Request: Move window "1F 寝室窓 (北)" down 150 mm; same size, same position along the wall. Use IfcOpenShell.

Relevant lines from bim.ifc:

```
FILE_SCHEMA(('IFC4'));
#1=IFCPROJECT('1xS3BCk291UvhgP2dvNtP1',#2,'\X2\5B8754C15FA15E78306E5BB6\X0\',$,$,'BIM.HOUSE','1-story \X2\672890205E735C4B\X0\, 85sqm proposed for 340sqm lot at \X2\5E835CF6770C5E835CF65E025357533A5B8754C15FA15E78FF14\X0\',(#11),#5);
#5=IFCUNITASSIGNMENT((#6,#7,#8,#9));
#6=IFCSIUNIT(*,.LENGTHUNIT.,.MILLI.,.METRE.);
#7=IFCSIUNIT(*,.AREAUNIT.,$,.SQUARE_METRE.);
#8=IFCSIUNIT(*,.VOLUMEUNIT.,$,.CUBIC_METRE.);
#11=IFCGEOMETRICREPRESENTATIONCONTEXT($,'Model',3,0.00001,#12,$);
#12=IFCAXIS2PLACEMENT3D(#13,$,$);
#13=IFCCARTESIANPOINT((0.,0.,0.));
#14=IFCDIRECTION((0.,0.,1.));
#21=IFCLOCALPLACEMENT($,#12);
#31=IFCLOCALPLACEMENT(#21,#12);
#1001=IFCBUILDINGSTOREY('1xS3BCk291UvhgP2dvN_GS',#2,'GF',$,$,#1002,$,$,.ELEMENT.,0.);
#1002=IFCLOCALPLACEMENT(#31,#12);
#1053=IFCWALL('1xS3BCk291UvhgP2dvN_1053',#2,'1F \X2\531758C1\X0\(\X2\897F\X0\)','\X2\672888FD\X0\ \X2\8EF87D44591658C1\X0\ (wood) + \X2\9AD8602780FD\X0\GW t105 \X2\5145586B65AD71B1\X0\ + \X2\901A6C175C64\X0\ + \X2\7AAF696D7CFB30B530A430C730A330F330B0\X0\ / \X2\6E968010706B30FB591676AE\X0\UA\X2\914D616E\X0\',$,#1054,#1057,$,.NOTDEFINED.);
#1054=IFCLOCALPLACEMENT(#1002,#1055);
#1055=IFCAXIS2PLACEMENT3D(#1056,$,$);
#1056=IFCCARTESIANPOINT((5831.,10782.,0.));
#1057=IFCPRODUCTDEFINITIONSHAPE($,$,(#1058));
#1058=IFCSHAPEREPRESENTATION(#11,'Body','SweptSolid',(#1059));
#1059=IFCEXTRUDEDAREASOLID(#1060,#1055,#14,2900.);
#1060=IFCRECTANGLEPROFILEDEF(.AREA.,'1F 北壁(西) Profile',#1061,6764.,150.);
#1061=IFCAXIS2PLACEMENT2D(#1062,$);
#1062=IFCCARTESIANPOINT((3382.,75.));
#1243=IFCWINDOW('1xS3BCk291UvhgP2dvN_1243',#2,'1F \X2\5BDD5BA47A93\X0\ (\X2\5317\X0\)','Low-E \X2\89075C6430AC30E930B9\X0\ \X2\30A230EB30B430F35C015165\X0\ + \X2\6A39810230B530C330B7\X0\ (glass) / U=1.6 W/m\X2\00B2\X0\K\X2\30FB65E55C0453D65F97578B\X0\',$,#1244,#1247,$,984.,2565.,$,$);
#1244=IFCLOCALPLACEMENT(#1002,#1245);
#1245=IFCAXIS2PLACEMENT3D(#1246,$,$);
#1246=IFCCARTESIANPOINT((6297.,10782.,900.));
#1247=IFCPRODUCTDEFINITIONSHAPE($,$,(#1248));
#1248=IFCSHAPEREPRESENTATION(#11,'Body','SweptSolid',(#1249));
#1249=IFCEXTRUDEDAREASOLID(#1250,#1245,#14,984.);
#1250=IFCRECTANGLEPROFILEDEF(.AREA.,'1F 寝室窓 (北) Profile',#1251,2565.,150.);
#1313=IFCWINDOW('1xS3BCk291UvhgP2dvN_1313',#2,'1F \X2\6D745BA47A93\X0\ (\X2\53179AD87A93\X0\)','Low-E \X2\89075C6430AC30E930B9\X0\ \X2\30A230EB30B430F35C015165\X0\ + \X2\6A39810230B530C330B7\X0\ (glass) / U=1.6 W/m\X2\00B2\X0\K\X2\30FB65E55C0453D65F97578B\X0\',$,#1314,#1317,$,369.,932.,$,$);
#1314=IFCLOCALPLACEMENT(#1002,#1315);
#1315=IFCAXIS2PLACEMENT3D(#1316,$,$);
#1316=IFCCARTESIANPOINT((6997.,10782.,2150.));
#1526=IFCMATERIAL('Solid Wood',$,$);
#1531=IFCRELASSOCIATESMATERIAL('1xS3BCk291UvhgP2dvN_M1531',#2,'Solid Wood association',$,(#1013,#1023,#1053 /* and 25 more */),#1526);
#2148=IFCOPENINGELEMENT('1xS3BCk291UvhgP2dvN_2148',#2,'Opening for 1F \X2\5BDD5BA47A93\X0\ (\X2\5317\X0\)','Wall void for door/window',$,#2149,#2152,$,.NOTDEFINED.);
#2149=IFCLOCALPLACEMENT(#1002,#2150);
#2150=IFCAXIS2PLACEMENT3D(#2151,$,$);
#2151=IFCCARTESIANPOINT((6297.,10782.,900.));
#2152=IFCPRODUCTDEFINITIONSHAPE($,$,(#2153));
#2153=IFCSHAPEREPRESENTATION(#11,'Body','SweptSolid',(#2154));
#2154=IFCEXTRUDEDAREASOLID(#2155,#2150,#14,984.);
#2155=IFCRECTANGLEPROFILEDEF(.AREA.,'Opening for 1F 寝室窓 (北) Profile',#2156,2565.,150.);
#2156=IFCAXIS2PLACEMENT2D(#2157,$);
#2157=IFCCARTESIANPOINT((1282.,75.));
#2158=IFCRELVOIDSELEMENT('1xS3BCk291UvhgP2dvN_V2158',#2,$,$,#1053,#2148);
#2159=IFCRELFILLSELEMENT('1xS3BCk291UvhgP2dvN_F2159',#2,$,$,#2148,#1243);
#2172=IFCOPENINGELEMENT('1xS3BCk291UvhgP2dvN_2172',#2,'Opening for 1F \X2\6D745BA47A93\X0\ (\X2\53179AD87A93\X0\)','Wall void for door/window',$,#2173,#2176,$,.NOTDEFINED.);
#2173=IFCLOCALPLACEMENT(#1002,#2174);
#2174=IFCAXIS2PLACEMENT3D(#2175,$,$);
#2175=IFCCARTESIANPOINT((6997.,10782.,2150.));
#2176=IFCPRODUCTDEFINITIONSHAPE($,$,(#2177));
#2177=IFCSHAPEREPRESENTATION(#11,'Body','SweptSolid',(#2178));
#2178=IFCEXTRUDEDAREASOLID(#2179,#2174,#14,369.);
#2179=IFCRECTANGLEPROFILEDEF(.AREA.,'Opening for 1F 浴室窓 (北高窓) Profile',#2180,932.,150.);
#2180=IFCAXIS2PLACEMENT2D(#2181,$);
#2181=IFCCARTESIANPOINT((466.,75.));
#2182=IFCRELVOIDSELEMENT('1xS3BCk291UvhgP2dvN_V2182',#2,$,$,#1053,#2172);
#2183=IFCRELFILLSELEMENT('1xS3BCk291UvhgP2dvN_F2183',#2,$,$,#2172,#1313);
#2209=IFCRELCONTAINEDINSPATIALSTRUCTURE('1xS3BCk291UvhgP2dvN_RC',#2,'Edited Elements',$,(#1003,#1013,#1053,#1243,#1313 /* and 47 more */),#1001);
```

```python
import numpy as np
import ifcopenshell
import ifcopenshell.api.geometry
import ifcopenshell.util.placement
import ifcopenshell.util.unit

model = ifcopenshell.open("bim.ifc")
unit_scale = ifcopenshell.util.unit.calculate_unit_scale(model)

window = model.by_guid("1xS3BCk291UvhgP2dvN_1243")
opening = window.FillsVoids[0].RelatingOpeningElement
dz = -150.0

shift = np.array([0.0, 0.0, dz])
# The window is not placed relative to its opening, so move both.
for product in (opening, window):
    matrix = ifcopenshell.util.placement.get_local_placement(product.ObjectPlacement)
    matrix[:3, 3] += shift
    ifcopenshell.api.geometry.edit_object_placement(model, product=product, matrix=matrix, is_si=False)

print(f"moved by {dz * unit_scale:+.3f} m")

model.write("bim_updated.ifc")
```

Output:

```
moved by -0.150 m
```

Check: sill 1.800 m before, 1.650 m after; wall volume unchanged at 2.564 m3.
